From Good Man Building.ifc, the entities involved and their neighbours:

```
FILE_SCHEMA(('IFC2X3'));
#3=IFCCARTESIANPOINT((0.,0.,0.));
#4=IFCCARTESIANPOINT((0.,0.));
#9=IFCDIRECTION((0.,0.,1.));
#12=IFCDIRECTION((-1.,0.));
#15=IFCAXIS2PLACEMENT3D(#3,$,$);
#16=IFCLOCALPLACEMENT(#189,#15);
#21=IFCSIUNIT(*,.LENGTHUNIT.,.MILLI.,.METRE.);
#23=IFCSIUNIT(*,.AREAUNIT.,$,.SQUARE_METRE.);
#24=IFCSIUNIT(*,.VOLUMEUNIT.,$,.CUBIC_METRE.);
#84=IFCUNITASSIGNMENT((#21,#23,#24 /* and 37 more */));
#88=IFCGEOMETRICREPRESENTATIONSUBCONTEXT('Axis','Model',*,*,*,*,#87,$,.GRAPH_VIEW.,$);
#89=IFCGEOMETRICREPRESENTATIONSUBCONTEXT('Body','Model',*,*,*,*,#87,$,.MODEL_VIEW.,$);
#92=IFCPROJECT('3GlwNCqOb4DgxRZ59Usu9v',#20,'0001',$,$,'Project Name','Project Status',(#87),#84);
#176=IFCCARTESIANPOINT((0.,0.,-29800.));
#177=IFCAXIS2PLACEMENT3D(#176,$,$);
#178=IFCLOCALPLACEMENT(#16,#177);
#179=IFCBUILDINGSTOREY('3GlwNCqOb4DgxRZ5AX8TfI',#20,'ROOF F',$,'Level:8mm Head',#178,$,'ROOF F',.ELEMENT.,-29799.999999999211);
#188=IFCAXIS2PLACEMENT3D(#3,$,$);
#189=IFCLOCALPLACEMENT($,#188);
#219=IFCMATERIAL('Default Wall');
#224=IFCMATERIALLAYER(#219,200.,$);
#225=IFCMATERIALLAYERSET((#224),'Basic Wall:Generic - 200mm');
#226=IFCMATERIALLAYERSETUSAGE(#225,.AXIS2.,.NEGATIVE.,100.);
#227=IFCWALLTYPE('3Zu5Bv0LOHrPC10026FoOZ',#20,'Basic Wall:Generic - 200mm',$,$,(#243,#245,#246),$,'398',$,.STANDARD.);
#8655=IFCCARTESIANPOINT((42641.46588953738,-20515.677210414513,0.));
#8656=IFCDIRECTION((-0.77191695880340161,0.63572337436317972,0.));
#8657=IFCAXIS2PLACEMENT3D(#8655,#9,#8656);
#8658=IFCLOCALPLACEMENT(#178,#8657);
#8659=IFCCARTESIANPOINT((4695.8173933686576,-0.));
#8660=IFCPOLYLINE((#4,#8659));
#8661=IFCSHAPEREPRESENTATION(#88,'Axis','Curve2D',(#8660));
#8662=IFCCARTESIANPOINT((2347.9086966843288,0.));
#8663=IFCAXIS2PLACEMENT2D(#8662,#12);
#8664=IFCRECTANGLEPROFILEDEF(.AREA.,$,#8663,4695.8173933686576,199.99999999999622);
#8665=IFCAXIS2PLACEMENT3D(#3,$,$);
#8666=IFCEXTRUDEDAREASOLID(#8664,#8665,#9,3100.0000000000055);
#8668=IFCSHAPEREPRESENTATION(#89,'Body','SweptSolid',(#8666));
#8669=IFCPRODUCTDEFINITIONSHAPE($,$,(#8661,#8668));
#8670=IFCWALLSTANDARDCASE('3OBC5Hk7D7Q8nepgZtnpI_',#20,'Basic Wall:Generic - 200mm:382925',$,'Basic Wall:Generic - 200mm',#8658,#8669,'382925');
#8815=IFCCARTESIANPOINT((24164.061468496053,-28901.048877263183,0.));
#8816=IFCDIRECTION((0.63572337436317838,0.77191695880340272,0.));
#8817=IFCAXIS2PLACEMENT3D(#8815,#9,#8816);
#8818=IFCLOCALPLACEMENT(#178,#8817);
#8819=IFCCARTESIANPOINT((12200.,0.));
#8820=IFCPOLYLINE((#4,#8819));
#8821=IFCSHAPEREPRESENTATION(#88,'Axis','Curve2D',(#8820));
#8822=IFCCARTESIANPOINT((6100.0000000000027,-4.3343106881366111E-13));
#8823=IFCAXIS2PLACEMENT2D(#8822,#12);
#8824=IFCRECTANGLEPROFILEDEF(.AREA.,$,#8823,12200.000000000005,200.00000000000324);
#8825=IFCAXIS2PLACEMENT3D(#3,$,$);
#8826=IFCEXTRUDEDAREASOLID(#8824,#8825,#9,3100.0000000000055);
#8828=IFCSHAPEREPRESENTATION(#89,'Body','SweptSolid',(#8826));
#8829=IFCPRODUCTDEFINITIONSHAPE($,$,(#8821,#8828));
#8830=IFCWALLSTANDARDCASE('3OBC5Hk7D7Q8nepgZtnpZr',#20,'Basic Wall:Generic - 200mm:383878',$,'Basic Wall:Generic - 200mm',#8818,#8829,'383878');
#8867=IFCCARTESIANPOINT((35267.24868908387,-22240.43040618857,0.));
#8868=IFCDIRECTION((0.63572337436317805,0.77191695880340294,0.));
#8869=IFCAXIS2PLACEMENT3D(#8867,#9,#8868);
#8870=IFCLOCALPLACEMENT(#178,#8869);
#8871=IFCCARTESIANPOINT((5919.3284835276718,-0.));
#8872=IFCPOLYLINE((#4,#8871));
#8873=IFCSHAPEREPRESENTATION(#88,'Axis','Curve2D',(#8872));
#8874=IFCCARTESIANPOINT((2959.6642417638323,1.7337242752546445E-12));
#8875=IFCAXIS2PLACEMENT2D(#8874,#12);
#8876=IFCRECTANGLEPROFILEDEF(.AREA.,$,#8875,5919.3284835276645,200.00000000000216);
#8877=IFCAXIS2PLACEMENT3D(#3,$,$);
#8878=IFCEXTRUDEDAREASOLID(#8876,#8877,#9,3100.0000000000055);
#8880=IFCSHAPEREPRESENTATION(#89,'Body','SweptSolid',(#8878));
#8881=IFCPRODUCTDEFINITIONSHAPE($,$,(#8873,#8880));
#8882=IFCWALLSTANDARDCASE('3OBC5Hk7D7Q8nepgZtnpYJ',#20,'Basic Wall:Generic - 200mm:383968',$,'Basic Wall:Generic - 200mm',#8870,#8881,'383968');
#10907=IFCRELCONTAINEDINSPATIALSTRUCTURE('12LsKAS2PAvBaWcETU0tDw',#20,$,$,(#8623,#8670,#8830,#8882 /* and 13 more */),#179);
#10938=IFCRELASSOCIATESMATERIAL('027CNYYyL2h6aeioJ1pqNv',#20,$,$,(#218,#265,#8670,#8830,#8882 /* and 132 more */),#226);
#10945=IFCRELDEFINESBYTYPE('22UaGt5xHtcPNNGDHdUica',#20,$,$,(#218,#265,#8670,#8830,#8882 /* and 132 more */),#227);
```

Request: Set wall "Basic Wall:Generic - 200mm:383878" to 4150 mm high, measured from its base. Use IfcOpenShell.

```python
import ifcopenshell
import ifcopenshell.geom
import ifcopenshell.util.representation
import ifcopenshell.util.shape
import ifcopenshell.util.unit

model = ifcopenshell.open("Good Man Building.ifc")
unit_scale = ifcopenshell.util.unit.calculate_unit_scale(model)
settings = ifcopenshell.geom.settings()


def volume(element):
    """Net volume in cubic metres, openings subtracted."""
    shape = ifcopenshell.geom.create_shape(settings, element)
    return ifcopenshell.util.shape.get_volume(shape.geometry)


wall = model.by_id(8830)
before = volume(wall)

body = ifcopenshell.util.representation.get_representation(wall, "Model", "Body")
solid = body.Items[0]
old_height = solid.Depth
solid.Depth = 4.15 / unit_scale
after = volume(wall)

print(f"height {old_height:g} -> {solid.Depth:g}, volume {before:.3f} -> {after:.3f} m3")

model.write("Good Man Building_rev.ifc")
```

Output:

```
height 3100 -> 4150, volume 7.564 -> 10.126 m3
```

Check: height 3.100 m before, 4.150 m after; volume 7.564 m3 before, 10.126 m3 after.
